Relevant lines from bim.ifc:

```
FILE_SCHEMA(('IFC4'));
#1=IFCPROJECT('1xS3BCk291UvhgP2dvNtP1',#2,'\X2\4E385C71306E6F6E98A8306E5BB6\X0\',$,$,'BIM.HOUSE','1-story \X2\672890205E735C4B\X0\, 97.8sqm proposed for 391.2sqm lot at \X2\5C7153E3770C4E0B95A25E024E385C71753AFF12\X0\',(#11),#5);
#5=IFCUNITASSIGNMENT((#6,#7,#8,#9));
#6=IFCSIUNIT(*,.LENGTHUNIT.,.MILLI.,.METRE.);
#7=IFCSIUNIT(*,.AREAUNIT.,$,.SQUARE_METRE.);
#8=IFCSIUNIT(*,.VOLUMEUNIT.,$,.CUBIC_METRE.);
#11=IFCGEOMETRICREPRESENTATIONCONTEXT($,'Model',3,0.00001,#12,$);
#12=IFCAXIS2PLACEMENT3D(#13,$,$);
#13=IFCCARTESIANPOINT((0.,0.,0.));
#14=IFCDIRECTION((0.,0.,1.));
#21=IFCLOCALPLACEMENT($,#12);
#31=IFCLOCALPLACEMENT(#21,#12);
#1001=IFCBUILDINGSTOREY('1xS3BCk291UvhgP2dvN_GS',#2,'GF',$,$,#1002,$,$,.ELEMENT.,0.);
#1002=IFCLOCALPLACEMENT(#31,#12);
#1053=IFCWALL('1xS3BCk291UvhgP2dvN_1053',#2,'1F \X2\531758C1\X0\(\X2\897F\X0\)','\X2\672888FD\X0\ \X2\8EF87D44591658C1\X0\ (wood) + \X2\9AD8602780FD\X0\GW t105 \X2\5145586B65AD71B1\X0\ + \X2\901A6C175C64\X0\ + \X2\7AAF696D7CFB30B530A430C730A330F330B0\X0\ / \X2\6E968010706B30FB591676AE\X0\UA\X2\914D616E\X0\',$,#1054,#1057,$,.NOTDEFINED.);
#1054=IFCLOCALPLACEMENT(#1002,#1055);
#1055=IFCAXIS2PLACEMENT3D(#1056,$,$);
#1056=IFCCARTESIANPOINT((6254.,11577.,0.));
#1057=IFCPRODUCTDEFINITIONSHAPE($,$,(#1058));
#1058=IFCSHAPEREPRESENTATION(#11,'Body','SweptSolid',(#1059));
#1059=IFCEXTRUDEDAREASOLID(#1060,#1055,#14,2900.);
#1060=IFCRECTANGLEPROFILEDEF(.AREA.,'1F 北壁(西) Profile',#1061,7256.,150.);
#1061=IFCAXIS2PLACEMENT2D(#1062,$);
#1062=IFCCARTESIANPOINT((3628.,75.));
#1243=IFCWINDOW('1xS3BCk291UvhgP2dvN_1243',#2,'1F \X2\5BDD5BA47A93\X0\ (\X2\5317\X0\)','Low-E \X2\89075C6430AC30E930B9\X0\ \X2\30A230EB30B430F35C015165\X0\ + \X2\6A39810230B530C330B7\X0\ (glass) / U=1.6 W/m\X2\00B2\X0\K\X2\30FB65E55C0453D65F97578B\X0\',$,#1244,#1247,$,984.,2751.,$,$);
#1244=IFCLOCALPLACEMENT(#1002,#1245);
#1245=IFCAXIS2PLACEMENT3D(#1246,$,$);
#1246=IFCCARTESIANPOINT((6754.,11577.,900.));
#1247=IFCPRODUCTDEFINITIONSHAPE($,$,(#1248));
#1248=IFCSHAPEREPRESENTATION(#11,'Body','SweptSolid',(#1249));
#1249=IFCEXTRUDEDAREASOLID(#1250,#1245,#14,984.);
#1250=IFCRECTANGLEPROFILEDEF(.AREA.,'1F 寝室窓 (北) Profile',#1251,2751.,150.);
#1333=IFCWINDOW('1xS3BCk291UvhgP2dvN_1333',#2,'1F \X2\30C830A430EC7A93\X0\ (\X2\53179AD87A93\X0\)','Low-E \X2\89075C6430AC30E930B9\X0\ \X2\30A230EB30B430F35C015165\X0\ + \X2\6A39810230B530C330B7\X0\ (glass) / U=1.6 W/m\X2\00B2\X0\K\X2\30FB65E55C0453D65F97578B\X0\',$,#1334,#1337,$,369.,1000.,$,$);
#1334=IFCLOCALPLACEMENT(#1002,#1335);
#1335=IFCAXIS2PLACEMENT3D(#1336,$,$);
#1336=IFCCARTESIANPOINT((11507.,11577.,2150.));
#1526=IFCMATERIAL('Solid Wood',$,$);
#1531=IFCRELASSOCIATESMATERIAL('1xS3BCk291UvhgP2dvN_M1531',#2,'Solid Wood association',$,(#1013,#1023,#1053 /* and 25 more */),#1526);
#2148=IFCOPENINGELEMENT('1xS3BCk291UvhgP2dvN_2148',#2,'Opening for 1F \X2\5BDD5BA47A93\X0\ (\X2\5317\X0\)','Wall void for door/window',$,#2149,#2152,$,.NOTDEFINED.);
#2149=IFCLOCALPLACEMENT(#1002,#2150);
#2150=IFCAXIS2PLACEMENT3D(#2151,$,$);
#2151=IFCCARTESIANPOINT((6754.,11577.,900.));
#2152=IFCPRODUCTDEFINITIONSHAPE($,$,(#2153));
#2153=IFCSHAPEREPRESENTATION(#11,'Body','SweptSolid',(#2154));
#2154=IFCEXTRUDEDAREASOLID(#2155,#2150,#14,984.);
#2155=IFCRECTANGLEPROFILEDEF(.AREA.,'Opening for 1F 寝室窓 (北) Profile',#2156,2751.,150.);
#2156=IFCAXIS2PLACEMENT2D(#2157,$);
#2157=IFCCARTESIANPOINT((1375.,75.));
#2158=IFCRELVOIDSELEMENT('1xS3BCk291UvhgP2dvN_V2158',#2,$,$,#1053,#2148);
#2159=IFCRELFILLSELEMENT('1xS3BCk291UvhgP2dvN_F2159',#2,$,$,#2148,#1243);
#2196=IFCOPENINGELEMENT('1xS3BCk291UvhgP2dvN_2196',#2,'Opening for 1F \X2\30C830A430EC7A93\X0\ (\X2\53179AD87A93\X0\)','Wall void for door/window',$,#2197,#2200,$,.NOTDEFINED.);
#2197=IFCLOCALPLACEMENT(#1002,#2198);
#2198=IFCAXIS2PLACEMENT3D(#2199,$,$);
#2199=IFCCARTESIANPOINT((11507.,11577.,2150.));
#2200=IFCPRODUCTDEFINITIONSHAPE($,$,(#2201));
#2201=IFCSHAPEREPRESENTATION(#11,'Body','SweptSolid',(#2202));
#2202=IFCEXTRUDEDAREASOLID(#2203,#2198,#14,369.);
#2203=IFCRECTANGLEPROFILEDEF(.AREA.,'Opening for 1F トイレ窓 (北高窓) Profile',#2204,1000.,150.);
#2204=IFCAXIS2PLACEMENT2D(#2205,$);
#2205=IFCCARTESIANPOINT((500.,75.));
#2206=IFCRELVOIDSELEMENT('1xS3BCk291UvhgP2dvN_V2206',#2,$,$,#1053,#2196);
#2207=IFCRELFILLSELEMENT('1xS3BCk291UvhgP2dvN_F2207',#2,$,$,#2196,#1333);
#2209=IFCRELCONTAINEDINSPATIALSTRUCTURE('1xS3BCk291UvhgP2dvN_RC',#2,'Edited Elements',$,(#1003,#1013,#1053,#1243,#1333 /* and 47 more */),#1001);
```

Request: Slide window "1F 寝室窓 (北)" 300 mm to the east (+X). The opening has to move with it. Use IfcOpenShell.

```python
import ifcopenshell
import ifcopenshell.api.geometry
import ifcopenshell.util.placement
import ifcopenshell.util.unit

model = ifcopenshell.open("bim.ifc")
unit_scale = ifcopenshell.util.unit.calculate_unit_scale(model)

window = model.by_guid("1xS3BCk291UvhgP2dvN_1243")
opening = window.FillsVoids[0].RelatingOpeningElement
wall = opening.VoidsElements[0].RelatingBuildingElement

wall_matrix = ifcopenshell.util.placement.get_local_placement(wall.ObjectPlacement)
shift = wall_matrix[:3, 0] * 0.3 / unit_scale
before = ifcopenshell.util.placement.get_local_placement(window.ObjectPlacement)[:3, 3].copy()

# The window is not placed relative to its opening, so move both.
for product in (opening, window):
    matrix = ifcopenshell.util.placement.get_local_placement(product.ObjectPlacement)
    matrix[:3, 3] += shift
    ifcopenshell.api.geometry.edit_object_placement(model, product=product, matrix=matrix, is_si=False)

after = ifcopenshell.util.placement.get_local_placement(window.ObjectPlacement)[:3, 3]
print("window moved by", (after - before).round(3) + 0.0)

model.write("bim_updated.ifc")
```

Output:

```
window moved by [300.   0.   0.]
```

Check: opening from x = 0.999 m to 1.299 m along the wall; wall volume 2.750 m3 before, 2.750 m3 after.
